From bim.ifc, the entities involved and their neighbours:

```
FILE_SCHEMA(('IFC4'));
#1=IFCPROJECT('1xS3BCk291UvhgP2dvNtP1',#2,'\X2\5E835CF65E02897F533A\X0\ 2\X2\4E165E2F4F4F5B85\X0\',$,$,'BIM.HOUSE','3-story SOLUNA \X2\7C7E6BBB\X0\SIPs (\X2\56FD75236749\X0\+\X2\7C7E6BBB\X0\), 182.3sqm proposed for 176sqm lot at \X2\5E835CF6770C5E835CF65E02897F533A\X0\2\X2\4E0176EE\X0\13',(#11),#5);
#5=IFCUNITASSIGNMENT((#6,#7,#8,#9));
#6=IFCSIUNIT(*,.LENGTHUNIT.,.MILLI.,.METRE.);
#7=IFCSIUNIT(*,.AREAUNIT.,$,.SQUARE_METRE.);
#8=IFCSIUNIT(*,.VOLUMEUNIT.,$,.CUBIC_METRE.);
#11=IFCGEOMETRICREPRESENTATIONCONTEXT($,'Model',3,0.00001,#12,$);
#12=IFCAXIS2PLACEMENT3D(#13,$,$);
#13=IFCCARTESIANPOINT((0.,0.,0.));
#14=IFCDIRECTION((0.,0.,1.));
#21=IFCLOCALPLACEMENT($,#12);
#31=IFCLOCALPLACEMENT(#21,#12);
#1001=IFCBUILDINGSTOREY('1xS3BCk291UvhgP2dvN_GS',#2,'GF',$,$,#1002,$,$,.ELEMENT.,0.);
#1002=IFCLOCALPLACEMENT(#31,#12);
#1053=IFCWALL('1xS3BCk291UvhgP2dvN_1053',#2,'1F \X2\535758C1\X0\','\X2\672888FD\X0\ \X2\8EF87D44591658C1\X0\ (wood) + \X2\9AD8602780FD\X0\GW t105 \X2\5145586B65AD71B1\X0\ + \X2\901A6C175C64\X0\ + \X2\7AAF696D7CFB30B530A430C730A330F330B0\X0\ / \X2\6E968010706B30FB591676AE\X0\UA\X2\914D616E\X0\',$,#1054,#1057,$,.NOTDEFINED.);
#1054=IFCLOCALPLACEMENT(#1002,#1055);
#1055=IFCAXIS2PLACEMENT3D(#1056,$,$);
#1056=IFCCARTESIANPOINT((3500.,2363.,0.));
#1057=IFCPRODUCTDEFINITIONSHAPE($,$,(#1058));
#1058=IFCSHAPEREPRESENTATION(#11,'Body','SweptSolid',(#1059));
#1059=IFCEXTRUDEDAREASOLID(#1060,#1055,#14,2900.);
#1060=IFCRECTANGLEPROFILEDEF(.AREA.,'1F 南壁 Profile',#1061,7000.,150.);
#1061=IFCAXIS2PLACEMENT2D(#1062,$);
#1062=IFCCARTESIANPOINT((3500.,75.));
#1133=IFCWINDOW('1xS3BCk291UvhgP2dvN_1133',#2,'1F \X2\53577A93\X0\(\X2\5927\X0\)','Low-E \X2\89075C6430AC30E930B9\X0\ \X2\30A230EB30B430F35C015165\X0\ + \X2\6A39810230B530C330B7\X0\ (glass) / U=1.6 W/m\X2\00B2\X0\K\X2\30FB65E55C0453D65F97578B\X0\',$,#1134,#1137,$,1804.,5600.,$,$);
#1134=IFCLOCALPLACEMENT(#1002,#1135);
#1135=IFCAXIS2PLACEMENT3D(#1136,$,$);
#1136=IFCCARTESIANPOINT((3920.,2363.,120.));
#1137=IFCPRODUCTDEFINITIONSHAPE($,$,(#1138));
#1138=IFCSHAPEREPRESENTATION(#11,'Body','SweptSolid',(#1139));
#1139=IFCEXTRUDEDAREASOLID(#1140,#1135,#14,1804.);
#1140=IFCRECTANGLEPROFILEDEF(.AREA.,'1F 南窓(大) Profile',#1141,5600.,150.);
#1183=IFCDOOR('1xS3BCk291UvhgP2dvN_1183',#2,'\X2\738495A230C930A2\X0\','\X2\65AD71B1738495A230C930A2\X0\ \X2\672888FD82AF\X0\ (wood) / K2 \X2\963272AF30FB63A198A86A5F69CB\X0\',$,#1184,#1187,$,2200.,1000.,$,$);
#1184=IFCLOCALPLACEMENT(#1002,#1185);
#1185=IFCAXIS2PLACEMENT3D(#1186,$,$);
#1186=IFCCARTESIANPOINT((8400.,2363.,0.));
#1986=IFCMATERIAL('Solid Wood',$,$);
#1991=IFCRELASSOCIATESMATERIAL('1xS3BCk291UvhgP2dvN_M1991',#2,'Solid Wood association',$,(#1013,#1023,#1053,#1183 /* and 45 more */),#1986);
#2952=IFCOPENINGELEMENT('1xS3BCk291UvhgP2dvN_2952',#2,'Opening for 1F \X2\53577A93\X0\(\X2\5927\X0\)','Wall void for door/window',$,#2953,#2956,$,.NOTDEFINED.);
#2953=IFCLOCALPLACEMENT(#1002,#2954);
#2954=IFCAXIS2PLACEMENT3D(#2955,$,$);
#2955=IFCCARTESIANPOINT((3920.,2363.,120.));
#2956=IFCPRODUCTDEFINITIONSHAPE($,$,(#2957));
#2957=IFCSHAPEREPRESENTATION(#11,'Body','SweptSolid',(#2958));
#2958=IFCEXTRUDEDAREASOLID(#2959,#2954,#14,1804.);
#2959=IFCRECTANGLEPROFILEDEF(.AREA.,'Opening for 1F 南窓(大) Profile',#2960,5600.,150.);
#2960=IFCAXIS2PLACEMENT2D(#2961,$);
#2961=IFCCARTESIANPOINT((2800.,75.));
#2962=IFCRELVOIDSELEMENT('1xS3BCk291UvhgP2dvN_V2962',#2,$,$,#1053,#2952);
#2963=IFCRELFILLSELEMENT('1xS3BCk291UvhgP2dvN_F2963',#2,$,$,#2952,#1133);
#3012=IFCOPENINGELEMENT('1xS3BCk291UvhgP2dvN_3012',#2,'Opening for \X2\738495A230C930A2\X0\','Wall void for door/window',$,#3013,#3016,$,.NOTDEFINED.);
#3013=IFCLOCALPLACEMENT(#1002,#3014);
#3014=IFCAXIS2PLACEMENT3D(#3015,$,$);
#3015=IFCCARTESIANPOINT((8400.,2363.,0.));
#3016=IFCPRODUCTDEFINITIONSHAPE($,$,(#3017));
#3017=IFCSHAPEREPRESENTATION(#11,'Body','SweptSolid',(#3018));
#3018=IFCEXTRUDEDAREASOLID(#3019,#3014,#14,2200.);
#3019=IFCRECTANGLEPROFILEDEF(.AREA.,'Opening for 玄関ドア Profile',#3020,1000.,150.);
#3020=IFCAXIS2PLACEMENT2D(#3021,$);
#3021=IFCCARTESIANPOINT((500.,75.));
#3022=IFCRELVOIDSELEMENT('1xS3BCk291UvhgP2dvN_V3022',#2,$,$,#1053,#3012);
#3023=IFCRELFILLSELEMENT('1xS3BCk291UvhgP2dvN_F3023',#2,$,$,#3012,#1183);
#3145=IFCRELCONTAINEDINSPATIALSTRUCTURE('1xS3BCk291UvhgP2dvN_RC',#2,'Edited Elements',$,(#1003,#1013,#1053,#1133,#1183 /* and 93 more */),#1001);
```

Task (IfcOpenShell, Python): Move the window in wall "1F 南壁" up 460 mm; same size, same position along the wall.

```python
import numpy as np
import ifcopenshell
import ifcopenshell.api.geometry
import ifcopenshell.util.placement
import ifcopenshell.util.unit

model = ifcopenshell.open("bim.ifc")
unit_scale = ifcopenshell.util.unit.calculate_unit_scale(model)

window = model.by_id(1133)
opening = window.FillsVoids[0].RelatingOpeningElement
dz = 0.46 / unit_scale

shift = np.array([0.0, 0.0, dz])
# The window is not placed relative to its opening, so move both.
for product in (opening, window):
    matrix = ifcopenshell.util.placement.get_local_placement(product.ObjectPlacement)
    matrix[:3, 3] += shift
    ifcopenshell.api.geometry.edit_object_placement(model, product=product, matrix=matrix, is_si=False)

print(f"moved by {dz * unit_scale:+.3f} m")

model.write("bim_updated.ifc")
```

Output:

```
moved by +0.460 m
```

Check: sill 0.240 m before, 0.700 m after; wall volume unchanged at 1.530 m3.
